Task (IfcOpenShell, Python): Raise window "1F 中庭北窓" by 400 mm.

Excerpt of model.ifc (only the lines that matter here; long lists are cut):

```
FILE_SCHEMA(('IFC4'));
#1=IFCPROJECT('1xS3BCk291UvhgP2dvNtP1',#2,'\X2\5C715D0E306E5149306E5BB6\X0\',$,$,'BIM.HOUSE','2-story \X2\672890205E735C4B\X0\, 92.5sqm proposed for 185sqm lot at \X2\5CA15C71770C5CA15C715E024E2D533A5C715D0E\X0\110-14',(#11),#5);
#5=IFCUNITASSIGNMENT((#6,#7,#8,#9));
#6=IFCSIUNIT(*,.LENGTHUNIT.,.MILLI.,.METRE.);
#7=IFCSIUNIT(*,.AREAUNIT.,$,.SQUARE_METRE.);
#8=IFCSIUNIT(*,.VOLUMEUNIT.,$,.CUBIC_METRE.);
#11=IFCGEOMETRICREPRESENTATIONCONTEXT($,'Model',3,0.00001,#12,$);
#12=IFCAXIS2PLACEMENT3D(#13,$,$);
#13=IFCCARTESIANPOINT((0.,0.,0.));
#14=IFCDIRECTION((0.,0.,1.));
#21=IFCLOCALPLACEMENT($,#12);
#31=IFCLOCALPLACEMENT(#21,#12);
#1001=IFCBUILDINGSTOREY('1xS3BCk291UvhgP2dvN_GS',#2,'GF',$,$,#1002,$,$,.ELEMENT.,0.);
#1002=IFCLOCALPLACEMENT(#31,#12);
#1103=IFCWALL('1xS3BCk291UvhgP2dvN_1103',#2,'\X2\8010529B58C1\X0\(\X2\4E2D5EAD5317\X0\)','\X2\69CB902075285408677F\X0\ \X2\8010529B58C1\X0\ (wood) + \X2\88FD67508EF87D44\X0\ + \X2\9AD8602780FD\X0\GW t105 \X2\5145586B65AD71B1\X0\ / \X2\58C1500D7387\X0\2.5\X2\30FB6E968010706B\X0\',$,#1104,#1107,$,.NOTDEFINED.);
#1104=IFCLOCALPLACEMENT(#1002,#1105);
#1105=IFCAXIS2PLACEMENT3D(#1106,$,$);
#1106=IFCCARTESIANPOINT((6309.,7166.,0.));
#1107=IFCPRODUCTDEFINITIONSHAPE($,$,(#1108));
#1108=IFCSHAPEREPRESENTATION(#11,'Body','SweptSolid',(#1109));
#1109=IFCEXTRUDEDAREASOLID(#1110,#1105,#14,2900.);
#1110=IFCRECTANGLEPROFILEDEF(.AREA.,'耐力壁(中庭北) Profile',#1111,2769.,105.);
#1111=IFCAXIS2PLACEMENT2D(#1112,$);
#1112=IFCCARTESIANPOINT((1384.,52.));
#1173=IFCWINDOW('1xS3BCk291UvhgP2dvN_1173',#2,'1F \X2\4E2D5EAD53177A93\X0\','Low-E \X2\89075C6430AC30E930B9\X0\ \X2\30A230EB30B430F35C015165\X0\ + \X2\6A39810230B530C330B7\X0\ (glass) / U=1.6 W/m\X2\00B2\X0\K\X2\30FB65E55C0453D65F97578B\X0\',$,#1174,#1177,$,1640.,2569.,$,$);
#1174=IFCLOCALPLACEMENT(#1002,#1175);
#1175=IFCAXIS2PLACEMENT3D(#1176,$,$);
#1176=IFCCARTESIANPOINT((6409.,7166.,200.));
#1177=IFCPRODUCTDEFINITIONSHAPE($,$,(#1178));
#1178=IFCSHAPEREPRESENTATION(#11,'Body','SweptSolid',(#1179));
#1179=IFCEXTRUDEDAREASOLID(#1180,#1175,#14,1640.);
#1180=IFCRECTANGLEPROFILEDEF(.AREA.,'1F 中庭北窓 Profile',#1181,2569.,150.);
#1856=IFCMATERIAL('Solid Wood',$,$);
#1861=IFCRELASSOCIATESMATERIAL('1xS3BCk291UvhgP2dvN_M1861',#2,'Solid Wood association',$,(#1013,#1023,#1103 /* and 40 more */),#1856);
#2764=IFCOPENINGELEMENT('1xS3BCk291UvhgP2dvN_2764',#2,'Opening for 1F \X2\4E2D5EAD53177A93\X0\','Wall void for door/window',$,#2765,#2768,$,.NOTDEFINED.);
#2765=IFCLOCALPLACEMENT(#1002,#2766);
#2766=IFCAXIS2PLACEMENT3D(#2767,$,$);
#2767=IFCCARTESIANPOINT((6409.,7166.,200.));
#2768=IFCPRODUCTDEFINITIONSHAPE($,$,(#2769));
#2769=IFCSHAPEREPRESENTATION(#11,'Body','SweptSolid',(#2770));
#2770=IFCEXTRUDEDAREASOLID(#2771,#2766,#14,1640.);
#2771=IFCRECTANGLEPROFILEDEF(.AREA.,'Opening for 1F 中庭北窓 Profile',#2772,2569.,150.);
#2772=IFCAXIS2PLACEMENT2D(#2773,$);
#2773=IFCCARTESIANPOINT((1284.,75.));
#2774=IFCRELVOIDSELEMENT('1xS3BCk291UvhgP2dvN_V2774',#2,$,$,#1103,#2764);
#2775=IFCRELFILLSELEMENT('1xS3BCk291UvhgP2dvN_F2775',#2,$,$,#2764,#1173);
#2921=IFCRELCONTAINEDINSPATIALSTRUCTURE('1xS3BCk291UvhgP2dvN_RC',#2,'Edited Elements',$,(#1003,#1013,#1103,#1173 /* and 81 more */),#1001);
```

```python
import numpy as np
import ifcopenshell
import ifcopenshell.api.geometry
import ifcopenshell.util.placement
import ifcopenshell.util.unit

model = ifcopenshell.open("model.ifc")
unit_scale = ifcopenshell.util.unit.calculate_unit_scale(model)

window = model.by_guid("1xS3BCk291UvhgP2dvN_1173")
opening = window.FillsVoids[0].RelatingOpeningElement
dz = 0.4 / unit_scale

shift = np.array([0.0, 0.0, dz])
# The window is not placed relative to its opening, so move both.
for product in (opening, window):
    matrix = ifcopenshell.util.placement.get_local_placement(product.ObjectPlacement)
    matrix[:3, 3] += shift
    ifcopenshell.api.geometry.edit_object_placement(model, product=product, matrix=matrix, is_si=False)

print(f"moved by {dz * unit_scale:+.3f} m")

model.write("model_updated.ifc")
```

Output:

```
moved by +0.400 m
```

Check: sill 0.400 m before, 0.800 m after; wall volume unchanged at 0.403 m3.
